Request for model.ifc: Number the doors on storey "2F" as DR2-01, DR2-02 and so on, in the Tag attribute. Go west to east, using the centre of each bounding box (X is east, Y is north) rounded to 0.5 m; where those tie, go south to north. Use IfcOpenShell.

First a look at what the model holds.

```python
import ifcopenshell
import ifcopenshell.util.element
import ifcopenshell.util.placement

model = ifcopenshell.open("model.ifc")
print(model.schema)
storey = next(s for s in model.by_type("IfcBuildingStorey") if s.Name == "2F")
doors = [e for e in ifcopenshell.util.element.get_decomposition(storey) if e.is_a("IfcDoor")]
for e in sorted(doors, key=lambda e: e.id()):
    origin = ifcopenshell.util.placement.get_local_placement(e.ObjectPlacement)[:3, 3]
    print(e.id(), e.Tag, e.Name, origin.round(2) + 0.0, sep=" | ")
```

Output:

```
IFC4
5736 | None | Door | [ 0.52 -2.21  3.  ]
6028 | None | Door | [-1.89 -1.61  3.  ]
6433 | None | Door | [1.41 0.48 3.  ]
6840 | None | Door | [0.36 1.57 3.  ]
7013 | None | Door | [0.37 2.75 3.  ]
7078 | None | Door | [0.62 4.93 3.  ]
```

```python
import ifcopenshell
import ifcopenshell.geom
import ifcopenshell.util.element
import ifcopenshell.util.shape

model = ifcopenshell.open("model.ifc")
settings = ifcopenshell.geom.settings()
settings.set("use-world-coords", True)


def centre(element):
    shape = ifcopenshell.geom.create_shape(settings, element)
    return ifcopenshell.util.shape.get_bbox_centroid(shape.geometry)


storey = next(s for s in model.by_type("IfcBuildingStorey") if s.Name == "2F")
doors = [e for e in ifcopenshell.util.element.get_decomposition(storey) if e.is_a("IfcDoor")]

# Insertion points can sit at a corner or the storey origin, so sort by the geometry (in metres).
centres = {e: centre(e) for e in doors}
doors.sort(key=lambda e: (round(centres[e][0] / 0.5), centres[e][1]))

for i, e in enumerate(doors, start=1):
    number = f"DR2-{i:02d}"
    e.Tag = number
    print(e.id(), number)

model.write("model_updated.ifc")
```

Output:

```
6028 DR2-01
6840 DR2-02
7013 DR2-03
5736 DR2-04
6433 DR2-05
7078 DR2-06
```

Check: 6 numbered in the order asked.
